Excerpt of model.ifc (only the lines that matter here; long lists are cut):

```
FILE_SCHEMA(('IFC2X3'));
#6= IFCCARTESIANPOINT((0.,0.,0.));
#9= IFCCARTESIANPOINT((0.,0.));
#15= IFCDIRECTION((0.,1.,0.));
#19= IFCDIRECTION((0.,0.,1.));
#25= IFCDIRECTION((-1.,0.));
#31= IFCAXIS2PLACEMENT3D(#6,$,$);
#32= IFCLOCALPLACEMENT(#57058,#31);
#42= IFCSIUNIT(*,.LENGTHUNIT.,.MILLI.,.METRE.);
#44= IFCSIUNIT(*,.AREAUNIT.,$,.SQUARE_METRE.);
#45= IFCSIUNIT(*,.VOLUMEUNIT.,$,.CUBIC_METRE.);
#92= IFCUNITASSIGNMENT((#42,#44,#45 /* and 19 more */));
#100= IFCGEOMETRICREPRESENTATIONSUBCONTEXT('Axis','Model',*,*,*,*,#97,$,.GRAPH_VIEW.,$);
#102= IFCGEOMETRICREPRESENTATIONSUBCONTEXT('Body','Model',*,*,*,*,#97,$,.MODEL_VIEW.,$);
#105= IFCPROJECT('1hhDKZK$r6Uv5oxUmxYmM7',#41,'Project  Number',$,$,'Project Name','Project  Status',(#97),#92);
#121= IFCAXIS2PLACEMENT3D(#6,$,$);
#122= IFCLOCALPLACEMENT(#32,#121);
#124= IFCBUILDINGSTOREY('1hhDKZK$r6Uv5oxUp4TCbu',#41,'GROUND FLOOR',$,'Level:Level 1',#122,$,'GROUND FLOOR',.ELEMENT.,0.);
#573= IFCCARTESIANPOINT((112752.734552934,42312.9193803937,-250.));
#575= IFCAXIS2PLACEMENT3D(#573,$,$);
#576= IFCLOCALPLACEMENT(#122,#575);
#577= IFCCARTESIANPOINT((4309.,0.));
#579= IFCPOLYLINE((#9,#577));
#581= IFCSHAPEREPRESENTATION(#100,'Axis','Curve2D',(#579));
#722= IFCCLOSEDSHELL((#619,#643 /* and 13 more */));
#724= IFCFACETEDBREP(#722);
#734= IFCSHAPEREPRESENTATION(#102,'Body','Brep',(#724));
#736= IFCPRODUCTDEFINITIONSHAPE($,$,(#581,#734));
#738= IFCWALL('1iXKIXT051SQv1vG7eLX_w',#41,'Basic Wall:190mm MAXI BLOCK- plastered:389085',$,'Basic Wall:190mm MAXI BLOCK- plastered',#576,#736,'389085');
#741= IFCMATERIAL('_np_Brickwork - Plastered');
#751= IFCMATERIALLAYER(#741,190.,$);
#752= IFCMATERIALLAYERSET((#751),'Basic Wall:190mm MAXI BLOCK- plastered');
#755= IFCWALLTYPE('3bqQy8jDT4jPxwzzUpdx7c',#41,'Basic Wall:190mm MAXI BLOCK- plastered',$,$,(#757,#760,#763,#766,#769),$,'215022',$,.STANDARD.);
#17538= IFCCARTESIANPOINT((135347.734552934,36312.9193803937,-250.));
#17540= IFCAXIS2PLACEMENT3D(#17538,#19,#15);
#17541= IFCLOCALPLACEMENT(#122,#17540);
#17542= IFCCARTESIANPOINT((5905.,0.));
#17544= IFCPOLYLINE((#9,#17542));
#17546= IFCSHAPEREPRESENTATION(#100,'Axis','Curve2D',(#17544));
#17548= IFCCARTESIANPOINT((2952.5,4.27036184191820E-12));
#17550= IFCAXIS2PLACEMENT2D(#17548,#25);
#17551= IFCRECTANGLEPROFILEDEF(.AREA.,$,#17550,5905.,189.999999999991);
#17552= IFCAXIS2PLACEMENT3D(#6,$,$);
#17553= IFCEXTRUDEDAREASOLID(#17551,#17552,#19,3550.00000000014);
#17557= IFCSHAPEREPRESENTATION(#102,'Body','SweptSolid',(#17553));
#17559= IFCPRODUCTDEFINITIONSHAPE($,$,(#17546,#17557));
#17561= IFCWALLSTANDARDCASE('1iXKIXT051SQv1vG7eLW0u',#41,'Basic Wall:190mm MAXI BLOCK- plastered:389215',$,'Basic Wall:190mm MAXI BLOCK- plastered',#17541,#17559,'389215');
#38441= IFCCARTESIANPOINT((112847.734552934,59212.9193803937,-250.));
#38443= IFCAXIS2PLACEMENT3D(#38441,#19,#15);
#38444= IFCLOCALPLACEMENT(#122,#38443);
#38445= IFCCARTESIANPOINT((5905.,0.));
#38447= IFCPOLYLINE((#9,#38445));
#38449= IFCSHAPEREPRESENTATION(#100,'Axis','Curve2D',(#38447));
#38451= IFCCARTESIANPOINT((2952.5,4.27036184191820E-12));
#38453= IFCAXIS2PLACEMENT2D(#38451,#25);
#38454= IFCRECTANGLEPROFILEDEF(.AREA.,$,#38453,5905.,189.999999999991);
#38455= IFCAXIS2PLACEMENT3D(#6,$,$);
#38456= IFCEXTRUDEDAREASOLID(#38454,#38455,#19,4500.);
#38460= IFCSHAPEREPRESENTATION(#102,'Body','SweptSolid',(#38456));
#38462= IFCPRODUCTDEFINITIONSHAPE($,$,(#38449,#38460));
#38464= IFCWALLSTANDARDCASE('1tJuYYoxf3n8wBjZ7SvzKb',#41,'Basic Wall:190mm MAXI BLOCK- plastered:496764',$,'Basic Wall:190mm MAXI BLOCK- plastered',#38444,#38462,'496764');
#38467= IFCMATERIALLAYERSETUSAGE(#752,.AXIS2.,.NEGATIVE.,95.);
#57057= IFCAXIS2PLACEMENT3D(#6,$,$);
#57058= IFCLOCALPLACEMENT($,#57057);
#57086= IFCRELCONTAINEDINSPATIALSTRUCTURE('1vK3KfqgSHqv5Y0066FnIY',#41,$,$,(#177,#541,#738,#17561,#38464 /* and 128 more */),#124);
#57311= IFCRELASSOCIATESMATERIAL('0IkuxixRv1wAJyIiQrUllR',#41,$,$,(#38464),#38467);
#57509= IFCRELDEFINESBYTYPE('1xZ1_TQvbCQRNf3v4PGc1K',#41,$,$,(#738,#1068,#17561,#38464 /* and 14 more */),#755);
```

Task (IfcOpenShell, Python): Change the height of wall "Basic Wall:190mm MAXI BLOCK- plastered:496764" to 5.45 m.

```python
import ifcopenshell
import ifcopenshell.geom
import ifcopenshell.util.representation
import ifcopenshell.util.shape

model = ifcopenshell.open("model.ifc")
settings = ifcopenshell.geom.settings()


def volume(element):
    """Net volume in cubic metres, openings subtracted."""
    shape = ifcopenshell.geom.create_shape(settings, element)
    return ifcopenshell.util.shape.get_volume(shape.geometry)


wall = model.by_guid("1tJuYYoxf3n8wBjZ7SvzKb")
before = volume(wall)

body = ifcopenshell.util.representation.get_representation(wall, "Model", "Body")
solid = body.Items[0]
old_height = solid.Depth
solid.Depth = 5450.0
after = volume(wall)

print(f"height {old_height:g} -> {solid.Depth:g}, volume {before:.3f} -> {after:.3f} m3")

model.write("model_edited.ifc")
```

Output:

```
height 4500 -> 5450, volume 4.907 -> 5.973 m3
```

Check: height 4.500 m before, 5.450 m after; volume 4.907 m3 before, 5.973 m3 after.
